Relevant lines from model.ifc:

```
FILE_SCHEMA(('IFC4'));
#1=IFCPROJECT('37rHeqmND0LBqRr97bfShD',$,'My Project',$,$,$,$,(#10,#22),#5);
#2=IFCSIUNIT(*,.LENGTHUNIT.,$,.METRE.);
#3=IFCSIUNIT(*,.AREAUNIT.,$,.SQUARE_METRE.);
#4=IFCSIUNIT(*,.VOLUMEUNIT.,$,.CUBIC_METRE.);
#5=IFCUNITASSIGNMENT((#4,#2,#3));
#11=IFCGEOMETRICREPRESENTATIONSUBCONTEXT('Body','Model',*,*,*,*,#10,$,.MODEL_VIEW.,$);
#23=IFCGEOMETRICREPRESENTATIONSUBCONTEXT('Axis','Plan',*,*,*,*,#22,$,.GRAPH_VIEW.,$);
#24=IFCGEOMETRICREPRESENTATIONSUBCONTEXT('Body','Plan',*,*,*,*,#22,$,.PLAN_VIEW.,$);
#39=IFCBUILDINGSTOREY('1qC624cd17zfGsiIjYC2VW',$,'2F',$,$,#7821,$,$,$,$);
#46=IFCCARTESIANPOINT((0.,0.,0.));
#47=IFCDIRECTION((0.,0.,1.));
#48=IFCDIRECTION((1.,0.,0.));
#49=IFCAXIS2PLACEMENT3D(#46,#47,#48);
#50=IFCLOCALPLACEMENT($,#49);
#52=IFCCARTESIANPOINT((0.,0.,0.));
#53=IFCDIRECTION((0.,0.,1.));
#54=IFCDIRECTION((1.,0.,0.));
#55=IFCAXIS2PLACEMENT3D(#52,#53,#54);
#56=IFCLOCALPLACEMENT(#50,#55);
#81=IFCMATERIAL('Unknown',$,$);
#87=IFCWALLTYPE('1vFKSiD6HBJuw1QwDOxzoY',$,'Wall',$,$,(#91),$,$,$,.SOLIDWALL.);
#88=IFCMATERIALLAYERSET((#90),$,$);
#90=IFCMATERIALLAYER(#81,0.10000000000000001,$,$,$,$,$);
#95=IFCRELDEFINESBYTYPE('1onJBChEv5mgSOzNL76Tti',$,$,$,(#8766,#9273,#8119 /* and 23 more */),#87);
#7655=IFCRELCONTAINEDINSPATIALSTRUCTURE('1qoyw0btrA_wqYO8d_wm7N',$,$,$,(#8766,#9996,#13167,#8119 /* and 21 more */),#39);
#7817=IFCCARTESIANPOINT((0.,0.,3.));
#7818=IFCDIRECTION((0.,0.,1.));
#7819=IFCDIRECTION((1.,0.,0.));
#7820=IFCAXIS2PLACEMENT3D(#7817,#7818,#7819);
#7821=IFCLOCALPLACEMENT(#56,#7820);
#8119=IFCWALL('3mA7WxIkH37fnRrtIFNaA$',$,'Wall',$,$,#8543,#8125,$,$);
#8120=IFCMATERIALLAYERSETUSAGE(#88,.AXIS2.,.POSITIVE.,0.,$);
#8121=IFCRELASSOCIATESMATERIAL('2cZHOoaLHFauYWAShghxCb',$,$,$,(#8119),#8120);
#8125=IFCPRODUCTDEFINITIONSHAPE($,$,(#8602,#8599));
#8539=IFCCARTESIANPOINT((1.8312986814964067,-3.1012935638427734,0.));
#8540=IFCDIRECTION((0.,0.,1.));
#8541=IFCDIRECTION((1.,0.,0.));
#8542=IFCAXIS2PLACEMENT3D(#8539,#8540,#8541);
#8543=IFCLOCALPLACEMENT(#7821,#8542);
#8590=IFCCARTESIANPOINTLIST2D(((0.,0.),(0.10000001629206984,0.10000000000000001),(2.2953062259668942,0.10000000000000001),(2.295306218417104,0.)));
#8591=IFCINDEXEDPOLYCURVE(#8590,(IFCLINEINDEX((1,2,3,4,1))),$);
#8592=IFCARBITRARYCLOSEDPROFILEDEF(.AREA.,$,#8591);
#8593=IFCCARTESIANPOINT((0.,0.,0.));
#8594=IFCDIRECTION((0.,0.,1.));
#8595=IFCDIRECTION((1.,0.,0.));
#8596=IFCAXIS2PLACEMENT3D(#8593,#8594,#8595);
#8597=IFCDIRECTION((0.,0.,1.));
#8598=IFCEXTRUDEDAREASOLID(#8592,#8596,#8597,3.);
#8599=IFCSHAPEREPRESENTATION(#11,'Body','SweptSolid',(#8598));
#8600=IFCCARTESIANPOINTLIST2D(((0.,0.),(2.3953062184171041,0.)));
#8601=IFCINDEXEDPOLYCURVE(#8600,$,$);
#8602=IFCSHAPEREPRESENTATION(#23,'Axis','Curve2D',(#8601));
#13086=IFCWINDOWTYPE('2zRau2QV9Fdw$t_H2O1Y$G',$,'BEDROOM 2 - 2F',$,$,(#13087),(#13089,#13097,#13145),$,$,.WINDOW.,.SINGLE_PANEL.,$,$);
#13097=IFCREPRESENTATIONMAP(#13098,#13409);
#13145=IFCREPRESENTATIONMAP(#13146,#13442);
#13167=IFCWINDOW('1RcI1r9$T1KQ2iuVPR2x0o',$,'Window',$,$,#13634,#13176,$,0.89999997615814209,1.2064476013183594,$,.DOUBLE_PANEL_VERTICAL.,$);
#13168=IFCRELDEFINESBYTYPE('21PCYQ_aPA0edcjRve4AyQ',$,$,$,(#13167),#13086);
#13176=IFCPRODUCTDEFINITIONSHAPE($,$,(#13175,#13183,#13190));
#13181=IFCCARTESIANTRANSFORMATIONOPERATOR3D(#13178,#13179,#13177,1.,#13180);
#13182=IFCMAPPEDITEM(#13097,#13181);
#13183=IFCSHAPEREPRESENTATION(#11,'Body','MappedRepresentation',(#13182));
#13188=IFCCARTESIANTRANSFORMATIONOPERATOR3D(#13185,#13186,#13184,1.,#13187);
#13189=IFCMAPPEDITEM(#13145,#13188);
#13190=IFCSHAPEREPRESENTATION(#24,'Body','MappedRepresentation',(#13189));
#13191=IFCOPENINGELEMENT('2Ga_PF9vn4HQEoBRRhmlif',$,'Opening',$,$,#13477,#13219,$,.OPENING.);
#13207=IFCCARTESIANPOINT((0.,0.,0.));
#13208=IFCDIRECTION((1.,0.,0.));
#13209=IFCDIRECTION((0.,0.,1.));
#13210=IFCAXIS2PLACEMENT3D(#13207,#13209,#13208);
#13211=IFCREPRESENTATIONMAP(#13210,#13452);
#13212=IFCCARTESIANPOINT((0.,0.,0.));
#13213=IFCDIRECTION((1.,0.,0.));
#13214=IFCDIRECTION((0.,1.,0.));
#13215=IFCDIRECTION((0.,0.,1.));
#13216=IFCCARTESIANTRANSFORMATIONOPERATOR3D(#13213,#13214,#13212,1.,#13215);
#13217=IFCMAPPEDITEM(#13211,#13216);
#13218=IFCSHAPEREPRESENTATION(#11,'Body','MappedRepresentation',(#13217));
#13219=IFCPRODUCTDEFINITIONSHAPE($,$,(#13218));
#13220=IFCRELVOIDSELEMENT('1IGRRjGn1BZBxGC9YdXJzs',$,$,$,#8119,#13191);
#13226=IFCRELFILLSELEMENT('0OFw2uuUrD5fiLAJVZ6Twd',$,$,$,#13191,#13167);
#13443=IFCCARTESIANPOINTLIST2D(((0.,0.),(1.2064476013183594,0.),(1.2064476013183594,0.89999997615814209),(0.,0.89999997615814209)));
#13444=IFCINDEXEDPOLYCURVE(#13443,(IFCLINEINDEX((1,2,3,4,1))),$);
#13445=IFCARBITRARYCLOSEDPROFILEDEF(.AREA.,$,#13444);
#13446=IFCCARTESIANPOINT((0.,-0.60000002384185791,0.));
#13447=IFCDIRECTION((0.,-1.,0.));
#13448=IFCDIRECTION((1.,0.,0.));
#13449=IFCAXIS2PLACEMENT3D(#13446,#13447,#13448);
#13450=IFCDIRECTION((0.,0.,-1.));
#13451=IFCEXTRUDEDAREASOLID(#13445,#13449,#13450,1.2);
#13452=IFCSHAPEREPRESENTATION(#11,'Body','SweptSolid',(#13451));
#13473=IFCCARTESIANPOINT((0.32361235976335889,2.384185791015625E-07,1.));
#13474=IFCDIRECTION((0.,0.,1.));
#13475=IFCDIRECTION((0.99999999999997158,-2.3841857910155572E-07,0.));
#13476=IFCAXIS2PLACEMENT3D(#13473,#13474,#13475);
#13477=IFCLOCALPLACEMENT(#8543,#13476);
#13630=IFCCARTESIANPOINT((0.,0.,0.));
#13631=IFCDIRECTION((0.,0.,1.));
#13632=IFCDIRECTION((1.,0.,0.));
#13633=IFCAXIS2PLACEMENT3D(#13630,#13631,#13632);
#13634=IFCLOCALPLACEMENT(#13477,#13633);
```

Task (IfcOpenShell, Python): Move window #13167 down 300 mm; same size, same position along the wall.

```python
import numpy as np
import ifcopenshell
import ifcopenshell.api.geometry
import ifcopenshell.util.placement
import ifcopenshell.util.unit

model = ifcopenshell.open("model.ifc")
unit_scale = ifcopenshell.util.unit.calculate_unit_scale(model)

window = model.by_id(13167)
opening = window.FillsVoids[0].RelatingOpeningElement
dz = -0.3 / unit_scale

shift = np.array([0.0, 0.0, dz])
# The window is placed relative to its opening, so it follows when the opening moves.
matrix = ifcopenshell.util.placement.get_local_placement(opening.ObjectPlacement)
matrix[:3, 3] += shift
ifcopenshell.api.geometry.edit_object_placement(
    model, product=opening, matrix=matrix, is_si=False, should_transform_children=True
)

print(f"moved by {dz * unit_scale:+.3f} m")

model.write("model_edited.ifc")
```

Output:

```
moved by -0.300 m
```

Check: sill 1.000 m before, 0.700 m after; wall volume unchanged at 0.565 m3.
